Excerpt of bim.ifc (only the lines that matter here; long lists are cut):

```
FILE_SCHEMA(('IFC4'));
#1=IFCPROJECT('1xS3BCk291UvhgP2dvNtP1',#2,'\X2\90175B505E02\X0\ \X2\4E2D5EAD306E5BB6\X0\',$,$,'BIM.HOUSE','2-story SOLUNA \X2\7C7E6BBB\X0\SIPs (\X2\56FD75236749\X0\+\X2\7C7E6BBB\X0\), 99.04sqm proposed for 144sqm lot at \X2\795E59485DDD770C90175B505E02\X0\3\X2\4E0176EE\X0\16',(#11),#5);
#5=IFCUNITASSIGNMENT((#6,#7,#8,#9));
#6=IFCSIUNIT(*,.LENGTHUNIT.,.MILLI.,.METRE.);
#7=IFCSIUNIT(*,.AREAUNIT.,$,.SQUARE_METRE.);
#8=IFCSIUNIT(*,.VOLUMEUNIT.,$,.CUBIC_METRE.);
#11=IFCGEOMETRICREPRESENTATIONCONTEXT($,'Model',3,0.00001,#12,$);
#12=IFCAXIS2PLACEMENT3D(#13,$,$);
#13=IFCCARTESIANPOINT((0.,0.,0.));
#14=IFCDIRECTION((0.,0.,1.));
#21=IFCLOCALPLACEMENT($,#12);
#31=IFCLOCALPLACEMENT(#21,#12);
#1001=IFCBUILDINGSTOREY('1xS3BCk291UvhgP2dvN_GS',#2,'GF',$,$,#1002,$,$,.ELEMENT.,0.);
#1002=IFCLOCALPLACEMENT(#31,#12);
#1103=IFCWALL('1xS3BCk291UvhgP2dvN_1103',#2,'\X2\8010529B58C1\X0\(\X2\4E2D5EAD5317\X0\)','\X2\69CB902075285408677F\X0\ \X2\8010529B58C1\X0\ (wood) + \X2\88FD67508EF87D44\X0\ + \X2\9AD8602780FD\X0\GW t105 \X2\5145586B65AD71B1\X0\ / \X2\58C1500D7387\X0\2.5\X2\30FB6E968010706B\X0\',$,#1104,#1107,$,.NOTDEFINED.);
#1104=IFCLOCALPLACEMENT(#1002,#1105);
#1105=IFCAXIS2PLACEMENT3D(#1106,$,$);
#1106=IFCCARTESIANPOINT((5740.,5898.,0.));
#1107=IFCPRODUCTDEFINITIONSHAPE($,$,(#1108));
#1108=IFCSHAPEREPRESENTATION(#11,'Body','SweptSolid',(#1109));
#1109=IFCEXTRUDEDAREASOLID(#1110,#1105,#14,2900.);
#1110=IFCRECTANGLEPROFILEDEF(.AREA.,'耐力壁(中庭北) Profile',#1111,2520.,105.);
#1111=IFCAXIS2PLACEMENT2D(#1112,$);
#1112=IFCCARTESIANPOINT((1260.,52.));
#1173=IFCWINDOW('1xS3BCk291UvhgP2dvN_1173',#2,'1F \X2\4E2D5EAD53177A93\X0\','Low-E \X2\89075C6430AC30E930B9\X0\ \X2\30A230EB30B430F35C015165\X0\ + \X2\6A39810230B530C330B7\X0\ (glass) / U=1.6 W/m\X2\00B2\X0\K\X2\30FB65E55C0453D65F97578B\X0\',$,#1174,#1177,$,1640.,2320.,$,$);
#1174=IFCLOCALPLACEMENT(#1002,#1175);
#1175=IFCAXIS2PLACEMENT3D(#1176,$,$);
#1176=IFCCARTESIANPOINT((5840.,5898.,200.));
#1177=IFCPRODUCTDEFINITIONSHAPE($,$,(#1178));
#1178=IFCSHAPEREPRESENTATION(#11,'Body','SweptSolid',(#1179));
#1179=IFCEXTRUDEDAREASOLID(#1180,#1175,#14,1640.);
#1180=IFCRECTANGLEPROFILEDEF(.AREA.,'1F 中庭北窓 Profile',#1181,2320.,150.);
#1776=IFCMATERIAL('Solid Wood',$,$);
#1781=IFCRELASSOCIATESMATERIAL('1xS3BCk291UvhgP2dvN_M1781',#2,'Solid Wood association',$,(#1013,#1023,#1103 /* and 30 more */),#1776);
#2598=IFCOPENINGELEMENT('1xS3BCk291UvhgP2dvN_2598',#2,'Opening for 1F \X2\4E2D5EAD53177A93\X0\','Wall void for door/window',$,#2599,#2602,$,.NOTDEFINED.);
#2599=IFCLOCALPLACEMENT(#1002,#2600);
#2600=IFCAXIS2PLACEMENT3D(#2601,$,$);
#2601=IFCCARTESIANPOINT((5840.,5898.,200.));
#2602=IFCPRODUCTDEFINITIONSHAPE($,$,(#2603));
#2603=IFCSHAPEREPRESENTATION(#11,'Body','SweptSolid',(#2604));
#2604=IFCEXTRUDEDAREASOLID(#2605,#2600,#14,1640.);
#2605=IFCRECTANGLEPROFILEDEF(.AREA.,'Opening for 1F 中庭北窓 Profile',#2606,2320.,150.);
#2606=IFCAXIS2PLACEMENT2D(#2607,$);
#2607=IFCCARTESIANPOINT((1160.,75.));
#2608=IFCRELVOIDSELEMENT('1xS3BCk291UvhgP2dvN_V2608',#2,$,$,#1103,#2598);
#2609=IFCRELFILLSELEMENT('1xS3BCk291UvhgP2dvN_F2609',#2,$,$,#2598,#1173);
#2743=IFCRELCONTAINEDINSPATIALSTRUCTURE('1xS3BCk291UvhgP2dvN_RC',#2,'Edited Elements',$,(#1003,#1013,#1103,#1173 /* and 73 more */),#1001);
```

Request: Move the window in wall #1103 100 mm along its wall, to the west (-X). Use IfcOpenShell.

```python
import ifcopenshell
import ifcopenshell.api.geometry
import ifcopenshell.util.placement
import ifcopenshell.util.unit

model = ifcopenshell.open("bim.ifc")
unit_scale = ifcopenshell.util.unit.calculate_unit_scale(model)

window = model.by_guid("1xS3BCk291UvhgP2dvN_1173")
opening = window.FillsVoids[0].RelatingOpeningElement
wall = opening.VoidsElements[0].RelatingBuildingElement

wall_matrix = ifcopenshell.util.placement.get_local_placement(wall.ObjectPlacement)
shift = wall_matrix[:3, 0] * -0.1 / unit_scale
before = ifcopenshell.util.placement.get_local_placement(window.ObjectPlacement)[:3, 3].copy()

# The window is not placed relative to its opening, so move both.
for product in (opening, window):
    matrix = ifcopenshell.util.placement.get_local_placement(product.ObjectPlacement)
    matrix[:3, 3] += shift
    ifcopenshell.api.geometry.edit_object_placement(model, product=product, matrix=matrix, is_si=False)

after = ifcopenshell.util.placement.get_local_placement(window.ObjectPlacement)[:3, 3]
print("window moved by", (after - before).round(3) + 0.0)

model.write("bim_rev.ifc")
```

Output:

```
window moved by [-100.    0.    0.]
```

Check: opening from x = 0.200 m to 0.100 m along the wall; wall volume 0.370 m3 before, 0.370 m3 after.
